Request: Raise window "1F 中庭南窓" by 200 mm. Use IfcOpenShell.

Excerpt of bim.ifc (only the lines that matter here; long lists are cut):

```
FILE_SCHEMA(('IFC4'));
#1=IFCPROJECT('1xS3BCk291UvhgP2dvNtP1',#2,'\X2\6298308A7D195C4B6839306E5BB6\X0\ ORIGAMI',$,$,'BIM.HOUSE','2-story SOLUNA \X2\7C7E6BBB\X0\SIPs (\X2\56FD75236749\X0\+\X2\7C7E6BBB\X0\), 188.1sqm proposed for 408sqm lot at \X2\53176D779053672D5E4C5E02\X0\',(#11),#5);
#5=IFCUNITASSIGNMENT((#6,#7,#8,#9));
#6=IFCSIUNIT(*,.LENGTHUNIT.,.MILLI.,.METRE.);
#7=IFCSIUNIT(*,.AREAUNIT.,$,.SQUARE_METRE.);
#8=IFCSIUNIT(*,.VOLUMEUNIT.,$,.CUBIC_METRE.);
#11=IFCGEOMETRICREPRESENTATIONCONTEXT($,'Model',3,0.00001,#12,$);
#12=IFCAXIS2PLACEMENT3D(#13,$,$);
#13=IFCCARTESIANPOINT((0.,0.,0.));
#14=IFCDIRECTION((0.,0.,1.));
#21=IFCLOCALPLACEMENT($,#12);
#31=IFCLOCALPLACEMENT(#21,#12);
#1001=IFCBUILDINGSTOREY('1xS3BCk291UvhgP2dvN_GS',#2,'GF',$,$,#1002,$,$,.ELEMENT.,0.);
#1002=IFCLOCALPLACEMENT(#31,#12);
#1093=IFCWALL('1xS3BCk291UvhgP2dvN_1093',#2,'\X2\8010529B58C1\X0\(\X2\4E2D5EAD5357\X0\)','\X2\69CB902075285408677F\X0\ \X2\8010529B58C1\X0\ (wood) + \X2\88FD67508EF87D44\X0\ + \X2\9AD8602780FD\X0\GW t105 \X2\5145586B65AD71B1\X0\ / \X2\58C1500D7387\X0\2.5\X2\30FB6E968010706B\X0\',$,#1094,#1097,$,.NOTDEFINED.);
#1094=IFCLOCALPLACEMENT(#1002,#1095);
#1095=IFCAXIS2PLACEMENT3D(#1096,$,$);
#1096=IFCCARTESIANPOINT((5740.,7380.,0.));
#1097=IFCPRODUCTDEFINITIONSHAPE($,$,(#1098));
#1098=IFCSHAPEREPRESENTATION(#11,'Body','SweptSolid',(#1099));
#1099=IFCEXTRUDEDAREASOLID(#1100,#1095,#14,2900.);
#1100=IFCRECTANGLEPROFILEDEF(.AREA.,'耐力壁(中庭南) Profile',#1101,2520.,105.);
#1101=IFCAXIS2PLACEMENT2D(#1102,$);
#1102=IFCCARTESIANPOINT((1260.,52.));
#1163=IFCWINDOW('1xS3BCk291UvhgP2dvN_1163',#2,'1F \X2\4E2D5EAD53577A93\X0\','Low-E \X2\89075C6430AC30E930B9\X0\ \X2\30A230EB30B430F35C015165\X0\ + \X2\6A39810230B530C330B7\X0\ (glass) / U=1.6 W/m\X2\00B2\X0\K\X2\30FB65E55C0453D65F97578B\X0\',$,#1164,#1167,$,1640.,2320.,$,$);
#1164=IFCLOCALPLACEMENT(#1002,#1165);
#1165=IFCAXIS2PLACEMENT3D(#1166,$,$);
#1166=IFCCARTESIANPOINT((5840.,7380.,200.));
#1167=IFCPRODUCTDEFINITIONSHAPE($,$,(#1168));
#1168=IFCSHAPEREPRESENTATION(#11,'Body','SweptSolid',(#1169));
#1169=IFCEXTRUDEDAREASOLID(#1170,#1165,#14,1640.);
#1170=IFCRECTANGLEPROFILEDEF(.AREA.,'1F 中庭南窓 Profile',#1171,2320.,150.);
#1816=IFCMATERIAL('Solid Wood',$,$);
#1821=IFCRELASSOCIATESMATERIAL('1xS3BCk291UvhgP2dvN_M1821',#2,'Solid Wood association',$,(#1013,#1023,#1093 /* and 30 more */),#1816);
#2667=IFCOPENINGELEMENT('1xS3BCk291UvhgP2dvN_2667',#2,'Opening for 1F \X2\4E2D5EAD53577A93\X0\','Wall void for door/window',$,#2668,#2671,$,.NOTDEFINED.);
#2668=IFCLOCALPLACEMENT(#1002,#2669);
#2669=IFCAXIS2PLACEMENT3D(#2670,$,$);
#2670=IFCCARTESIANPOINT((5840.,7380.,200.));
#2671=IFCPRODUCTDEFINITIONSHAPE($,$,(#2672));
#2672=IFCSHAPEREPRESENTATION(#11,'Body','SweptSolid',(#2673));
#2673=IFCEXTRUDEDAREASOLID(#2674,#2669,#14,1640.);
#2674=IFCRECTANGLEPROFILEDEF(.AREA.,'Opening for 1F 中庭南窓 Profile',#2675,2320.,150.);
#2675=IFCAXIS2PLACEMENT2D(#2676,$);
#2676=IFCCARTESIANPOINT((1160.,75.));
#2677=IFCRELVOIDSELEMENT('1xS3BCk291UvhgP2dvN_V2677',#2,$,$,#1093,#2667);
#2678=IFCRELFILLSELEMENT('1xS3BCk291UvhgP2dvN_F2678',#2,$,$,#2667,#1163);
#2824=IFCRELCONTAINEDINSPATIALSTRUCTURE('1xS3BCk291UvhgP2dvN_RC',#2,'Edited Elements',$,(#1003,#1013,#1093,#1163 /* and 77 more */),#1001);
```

```python
import numpy as np
import ifcopenshell
import ifcopenshell.api.geometry
import ifcopenshell.util.placement
import ifcopenshell.util.unit

model = ifcopenshell.open("bim.ifc")
unit_scale = ifcopenshell.util.unit.calculate_unit_scale(model)

window = model.by_guid("1xS3BCk291UvhgP2dvN_1163")
opening = window.FillsVoids[0].RelatingOpeningElement
dz = 0.2 / unit_scale

shift = np.array([0.0, 0.0, dz])
# The window is not placed relative to its opening, so move both.
for product in (opening, window):
    matrix = ifcopenshell.util.placement.get_local_placement(product.ObjectPlacement)
    matrix[:3, 3] += shift
    ifcopenshell.api.geometry.edit_object_placement(model, product=product, matrix=matrix, is_si=False)

print(f"moved by {dz * unit_scale:+.3f} m")

model.write("bim_updated.ifc")
```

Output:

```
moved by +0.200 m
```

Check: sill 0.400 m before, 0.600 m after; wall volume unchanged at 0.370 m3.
